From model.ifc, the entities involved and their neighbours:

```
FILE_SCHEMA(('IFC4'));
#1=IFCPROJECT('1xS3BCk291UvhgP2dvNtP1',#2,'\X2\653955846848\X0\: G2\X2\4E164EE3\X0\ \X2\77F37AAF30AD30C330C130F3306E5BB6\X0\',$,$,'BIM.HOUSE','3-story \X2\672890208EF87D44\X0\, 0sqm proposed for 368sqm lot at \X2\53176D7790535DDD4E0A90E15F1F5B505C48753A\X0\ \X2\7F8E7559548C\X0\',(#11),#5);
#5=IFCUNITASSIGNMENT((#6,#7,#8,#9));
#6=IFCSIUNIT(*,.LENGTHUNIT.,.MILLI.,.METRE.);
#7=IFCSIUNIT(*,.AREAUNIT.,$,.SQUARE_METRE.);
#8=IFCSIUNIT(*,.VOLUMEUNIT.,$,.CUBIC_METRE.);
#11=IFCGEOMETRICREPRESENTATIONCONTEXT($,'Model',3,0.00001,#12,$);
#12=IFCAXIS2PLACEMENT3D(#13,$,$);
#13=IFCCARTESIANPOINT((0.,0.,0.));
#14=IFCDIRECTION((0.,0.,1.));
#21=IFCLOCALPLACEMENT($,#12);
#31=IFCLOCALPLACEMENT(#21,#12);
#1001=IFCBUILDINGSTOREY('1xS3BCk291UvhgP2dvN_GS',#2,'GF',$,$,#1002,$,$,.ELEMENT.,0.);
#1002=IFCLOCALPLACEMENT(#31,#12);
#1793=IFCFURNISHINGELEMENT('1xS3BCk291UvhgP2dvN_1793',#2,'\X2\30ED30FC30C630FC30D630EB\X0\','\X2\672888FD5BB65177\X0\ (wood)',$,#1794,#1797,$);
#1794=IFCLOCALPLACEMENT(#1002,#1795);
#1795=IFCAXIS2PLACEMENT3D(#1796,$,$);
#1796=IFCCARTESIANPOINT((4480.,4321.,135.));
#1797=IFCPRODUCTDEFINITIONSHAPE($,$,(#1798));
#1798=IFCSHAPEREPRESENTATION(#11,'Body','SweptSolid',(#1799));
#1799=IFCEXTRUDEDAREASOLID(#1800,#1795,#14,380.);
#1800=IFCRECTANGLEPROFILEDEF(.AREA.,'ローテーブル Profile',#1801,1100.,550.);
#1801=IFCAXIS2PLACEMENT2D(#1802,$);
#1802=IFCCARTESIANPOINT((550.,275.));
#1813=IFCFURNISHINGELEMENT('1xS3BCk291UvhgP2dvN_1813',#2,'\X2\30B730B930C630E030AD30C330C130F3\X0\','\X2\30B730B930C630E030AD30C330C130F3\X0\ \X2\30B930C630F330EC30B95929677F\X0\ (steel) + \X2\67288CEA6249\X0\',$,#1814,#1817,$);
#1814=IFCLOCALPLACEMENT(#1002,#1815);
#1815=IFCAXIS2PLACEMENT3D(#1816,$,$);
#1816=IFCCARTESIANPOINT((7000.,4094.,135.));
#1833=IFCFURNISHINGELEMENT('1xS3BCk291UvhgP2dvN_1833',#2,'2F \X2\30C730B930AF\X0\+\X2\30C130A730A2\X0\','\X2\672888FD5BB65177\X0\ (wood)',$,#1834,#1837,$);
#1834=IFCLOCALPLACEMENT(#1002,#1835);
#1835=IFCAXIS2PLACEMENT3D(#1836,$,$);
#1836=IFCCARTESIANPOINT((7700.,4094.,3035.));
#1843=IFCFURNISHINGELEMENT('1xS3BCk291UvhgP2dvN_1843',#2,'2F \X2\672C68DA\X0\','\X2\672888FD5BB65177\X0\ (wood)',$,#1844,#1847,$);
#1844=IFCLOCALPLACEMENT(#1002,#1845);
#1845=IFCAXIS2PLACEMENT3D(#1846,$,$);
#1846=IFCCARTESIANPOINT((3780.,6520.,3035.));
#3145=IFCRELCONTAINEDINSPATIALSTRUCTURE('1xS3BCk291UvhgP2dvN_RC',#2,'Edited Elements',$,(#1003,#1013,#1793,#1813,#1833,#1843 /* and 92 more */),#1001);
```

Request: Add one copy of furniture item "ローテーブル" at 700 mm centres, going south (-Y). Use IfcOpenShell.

```python
import numpy as np
import ifcopenshell
import ifcopenshell.api.geometry
import ifcopenshell.api.root
import ifcopenshell.util.element
import ifcopenshell.util.placement
import ifcopenshell.util.unit

model = ifcopenshell.open("model.ifc")
unit_scale = ifcopenshell.util.unit.calculate_unit_scale(model)


def reuse_history(source, copy):
    """copy_class also copies each property set's owner history, people and application; keep the originals."""
    for rel in copy.IsDefinedBy:
        if rel.is_a("IfcRelDefinesByProperties") and (history := rel.RelatingPropertyDefinition.OwnerHistory):
            rel.RelatingPropertyDefinition.OwnerHistory = source.OwnerHistory
            ifcopenshell.util.element.remove_deep2(model, history)


source = model.by_guid("1xS3BCk291UvhgP2dvN_1793")
base = ifcopenshell.util.placement.get_local_placement(source.ObjectPlacement)
step = np.array([0.0, -1.0, 0.0]) * 0.7 / unit_scale

for i in range(1, 2):
    copy = ifcopenshell.api.root.copy_class(model, product=source)
    copy.Representation = ifcopenshell.util.element.copy_deep(
        model, source.Representation, exclude=["IfcGeometricRepresentationContext", "IfcRepresentationMap"]
    )
    reuse_history(source, copy)
    matrix = base.copy()
    matrix[:3, 3] += i * step
    print("added at", matrix[:3, 3].round(3) + 0.0)
    ifcopenshell.api.geometry.edit_object_placement(model, product=copy, matrix=matrix, is_si=False)

model.write("model_v2.ifc")
```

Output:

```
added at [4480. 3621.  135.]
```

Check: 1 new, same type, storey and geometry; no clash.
